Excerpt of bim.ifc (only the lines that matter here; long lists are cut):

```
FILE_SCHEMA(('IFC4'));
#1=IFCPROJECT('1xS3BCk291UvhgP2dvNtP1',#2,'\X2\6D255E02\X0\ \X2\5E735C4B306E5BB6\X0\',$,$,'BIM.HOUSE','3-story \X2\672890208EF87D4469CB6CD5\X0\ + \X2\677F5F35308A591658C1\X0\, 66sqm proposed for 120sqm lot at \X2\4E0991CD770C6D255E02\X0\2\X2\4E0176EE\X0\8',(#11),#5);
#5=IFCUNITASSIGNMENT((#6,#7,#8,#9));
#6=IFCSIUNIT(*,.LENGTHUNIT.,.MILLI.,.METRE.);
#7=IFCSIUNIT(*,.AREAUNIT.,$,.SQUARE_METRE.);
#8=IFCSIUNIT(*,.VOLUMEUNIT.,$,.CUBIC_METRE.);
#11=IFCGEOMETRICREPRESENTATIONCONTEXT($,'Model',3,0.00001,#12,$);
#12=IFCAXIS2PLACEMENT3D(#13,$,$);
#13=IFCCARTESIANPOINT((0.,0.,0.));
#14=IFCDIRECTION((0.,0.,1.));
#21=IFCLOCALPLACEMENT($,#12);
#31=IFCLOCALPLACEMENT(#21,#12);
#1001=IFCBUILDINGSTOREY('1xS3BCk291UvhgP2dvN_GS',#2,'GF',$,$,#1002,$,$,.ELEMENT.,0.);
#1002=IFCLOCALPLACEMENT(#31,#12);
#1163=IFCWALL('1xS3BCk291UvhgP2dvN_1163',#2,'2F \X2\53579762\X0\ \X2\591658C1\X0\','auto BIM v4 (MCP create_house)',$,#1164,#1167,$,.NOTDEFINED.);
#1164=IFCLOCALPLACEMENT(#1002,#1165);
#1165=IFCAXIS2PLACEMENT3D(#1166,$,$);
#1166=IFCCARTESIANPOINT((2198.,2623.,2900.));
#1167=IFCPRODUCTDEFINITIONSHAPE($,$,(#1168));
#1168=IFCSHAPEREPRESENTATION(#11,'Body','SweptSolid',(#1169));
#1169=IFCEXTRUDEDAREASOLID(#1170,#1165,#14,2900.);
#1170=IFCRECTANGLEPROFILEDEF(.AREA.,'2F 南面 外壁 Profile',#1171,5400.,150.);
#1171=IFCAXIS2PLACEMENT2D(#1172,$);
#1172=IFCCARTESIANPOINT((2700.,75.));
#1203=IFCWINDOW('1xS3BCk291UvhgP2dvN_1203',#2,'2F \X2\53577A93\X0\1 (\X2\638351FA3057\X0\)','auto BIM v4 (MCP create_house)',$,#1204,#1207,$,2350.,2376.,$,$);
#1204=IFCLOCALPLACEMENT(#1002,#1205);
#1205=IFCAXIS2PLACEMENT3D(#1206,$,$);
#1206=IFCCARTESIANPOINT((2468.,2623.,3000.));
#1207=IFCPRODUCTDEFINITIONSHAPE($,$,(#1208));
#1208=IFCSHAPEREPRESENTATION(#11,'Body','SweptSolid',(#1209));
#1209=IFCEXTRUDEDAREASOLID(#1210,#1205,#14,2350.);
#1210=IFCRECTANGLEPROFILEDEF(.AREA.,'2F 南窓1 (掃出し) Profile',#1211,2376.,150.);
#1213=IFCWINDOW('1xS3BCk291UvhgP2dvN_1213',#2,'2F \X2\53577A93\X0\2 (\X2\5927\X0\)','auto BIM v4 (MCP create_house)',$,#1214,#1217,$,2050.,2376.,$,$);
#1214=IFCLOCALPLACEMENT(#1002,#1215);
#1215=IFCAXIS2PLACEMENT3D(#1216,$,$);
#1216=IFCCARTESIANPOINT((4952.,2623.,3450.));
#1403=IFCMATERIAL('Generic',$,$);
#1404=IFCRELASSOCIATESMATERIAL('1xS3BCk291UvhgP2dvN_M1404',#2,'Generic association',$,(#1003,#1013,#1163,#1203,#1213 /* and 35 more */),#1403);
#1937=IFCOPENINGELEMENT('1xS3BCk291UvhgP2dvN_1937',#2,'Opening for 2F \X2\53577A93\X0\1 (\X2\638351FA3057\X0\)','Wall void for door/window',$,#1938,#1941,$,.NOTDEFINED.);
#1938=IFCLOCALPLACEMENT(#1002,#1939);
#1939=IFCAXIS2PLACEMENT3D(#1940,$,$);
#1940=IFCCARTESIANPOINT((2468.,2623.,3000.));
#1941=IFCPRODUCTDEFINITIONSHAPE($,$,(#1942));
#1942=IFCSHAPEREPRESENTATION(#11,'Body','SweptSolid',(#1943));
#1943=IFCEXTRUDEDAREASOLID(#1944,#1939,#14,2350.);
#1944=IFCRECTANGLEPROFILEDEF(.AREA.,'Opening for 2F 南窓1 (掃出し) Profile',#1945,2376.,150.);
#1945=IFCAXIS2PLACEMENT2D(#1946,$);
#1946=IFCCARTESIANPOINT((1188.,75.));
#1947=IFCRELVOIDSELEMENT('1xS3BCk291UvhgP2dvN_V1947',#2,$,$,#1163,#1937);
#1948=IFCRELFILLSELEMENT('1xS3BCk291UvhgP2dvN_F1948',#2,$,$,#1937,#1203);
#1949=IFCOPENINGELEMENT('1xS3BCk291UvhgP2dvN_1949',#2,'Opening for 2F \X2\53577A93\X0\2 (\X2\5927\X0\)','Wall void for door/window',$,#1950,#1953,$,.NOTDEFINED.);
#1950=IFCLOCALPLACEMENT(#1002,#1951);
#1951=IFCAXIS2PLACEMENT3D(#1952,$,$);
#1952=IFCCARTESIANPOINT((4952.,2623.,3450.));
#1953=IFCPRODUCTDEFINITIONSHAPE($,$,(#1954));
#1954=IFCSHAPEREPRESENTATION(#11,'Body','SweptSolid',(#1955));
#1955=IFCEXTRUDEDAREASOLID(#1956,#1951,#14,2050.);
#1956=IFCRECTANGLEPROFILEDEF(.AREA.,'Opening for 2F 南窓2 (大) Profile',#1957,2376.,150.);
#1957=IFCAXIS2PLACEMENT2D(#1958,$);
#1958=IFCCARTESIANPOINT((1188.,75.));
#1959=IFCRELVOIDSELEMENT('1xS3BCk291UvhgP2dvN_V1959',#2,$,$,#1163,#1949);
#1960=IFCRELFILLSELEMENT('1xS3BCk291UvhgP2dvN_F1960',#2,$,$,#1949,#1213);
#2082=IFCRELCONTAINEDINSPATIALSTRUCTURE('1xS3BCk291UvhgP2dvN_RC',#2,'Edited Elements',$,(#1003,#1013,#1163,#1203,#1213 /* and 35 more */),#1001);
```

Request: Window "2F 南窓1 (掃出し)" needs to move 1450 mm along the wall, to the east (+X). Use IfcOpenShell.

```python
import ifcopenshell
import ifcopenshell.api.geometry
import ifcopenshell.util.placement
import ifcopenshell.util.unit

model = ifcopenshell.open("bim.ifc")
unit_scale = ifcopenshell.util.unit.calculate_unit_scale(model)

window = model.by_id(1203)
opening = window.FillsVoids[0].RelatingOpeningElement
wall = opening.VoidsElements[0].RelatingBuildingElement

wall_matrix = ifcopenshell.util.placement.get_local_placement(wall.ObjectPlacement)
shift = wall_matrix[:3, 0] * 1.45 / unit_scale
before = ifcopenshell.util.placement.get_local_placement(window.ObjectPlacement)[:3, 3].copy()

# The window is not placed relative to its opening, so move both.
for product in (opening, window):
    matrix = ifcopenshell.util.placement.get_local_placement(product.ObjectPlacement)
    matrix[:3, 3] += shift
    ifcopenshell.api.geometry.edit_object_placement(model, product=product, matrix=matrix, is_si=False)

after = ifcopenshell.util.placement.get_local_placement(window.ObjectPlacement)[:3, 3]
print("window moved by", (after - before).round(3) + 0.0)

model.write("bim_rev.ifc")
```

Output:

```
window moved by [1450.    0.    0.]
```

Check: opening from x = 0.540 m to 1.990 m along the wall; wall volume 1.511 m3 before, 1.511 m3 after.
